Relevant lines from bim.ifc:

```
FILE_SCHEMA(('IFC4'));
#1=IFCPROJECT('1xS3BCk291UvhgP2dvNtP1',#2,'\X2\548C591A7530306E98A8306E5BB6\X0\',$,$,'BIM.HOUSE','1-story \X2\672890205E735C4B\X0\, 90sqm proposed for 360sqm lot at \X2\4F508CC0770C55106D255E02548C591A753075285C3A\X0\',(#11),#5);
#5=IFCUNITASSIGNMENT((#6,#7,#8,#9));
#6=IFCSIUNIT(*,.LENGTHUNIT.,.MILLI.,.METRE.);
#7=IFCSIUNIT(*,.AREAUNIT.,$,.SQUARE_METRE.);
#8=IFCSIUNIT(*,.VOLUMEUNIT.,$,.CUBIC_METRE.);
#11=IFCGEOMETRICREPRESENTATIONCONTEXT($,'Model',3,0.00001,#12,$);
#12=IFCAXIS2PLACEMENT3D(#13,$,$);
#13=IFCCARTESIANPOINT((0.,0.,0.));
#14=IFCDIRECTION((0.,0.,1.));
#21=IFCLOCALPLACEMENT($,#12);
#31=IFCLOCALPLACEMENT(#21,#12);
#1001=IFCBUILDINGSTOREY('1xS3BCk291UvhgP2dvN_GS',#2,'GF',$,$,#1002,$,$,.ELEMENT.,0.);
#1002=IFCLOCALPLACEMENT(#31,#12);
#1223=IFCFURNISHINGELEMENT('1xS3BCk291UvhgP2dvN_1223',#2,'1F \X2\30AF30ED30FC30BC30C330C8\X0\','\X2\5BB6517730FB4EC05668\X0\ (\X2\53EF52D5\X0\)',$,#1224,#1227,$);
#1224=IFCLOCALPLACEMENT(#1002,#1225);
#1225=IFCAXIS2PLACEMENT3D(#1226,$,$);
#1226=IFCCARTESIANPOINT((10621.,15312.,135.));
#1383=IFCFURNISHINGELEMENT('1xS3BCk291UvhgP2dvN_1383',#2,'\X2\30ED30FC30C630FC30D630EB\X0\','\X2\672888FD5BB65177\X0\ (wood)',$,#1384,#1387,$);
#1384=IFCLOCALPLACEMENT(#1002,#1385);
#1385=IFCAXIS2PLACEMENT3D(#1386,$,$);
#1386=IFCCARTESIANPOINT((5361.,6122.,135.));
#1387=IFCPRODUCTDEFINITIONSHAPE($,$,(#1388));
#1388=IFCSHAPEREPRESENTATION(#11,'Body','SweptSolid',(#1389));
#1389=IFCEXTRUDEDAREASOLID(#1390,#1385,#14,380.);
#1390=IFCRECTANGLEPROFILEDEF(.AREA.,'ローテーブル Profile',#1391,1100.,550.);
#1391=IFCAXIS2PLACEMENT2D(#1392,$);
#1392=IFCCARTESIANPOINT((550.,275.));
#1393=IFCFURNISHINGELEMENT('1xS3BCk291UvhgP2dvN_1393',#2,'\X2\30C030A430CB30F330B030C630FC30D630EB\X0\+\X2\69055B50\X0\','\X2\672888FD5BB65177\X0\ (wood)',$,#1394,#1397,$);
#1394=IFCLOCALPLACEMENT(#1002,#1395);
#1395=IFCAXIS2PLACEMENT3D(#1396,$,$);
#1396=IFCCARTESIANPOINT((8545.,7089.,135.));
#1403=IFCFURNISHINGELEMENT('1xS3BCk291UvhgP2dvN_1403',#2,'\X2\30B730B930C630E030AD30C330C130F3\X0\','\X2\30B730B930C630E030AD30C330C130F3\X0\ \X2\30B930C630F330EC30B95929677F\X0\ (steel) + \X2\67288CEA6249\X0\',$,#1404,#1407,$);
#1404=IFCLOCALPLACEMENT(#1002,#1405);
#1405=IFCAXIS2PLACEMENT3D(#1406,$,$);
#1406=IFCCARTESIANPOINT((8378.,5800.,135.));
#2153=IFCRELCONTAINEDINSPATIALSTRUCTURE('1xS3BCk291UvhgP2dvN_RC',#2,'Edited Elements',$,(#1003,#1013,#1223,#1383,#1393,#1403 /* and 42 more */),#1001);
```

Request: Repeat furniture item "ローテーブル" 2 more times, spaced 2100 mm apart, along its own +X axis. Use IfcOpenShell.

```python
import ifcopenshell
import ifcopenshell.api.geometry
import ifcopenshell.api.root
import ifcopenshell.util.element
import ifcopenshell.util.placement
import ifcopenshell.util.unit

model = ifcopenshell.open("bim.ifc")
unit_scale = ifcopenshell.util.unit.calculate_unit_scale(model)


def reuse_history(source, copy):
    """copy_class also copies each property set's owner history, people and application; keep the originals."""
    for rel in copy.IsDefinedBy:
        if rel.is_a("IfcRelDefinesByProperties") and (history := rel.RelatingPropertyDefinition.OwnerHistory):
            rel.RelatingPropertyDefinition.OwnerHistory = source.OwnerHistory
            ifcopenshell.util.element.remove_deep2(model, history)


source = model.by_id(1383)
base = ifcopenshell.util.placement.get_local_placement(source.ObjectPlacement)
step = base[:3, 0] * 2.1 / unit_scale

for i in range(1, 3):
    copy = ifcopenshell.api.root.copy_class(model, product=source)
    copy.Representation = ifcopenshell.util.element.copy_deep(
        model, source.Representation, exclude=["IfcGeometricRepresentationContext", "IfcRepresentationMap"]
    )
    reuse_history(source, copy)
    matrix = base.copy()
    matrix[:3, 3] += i * step
    print("added at", matrix[:3, 3].round(3) + 0.0)
    ifcopenshell.api.geometry.edit_object_placement(model, product=copy, matrix=matrix, is_si=False)

model.write("bim_edited.ifc")
```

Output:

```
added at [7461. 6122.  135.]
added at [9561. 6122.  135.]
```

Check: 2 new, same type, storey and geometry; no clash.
